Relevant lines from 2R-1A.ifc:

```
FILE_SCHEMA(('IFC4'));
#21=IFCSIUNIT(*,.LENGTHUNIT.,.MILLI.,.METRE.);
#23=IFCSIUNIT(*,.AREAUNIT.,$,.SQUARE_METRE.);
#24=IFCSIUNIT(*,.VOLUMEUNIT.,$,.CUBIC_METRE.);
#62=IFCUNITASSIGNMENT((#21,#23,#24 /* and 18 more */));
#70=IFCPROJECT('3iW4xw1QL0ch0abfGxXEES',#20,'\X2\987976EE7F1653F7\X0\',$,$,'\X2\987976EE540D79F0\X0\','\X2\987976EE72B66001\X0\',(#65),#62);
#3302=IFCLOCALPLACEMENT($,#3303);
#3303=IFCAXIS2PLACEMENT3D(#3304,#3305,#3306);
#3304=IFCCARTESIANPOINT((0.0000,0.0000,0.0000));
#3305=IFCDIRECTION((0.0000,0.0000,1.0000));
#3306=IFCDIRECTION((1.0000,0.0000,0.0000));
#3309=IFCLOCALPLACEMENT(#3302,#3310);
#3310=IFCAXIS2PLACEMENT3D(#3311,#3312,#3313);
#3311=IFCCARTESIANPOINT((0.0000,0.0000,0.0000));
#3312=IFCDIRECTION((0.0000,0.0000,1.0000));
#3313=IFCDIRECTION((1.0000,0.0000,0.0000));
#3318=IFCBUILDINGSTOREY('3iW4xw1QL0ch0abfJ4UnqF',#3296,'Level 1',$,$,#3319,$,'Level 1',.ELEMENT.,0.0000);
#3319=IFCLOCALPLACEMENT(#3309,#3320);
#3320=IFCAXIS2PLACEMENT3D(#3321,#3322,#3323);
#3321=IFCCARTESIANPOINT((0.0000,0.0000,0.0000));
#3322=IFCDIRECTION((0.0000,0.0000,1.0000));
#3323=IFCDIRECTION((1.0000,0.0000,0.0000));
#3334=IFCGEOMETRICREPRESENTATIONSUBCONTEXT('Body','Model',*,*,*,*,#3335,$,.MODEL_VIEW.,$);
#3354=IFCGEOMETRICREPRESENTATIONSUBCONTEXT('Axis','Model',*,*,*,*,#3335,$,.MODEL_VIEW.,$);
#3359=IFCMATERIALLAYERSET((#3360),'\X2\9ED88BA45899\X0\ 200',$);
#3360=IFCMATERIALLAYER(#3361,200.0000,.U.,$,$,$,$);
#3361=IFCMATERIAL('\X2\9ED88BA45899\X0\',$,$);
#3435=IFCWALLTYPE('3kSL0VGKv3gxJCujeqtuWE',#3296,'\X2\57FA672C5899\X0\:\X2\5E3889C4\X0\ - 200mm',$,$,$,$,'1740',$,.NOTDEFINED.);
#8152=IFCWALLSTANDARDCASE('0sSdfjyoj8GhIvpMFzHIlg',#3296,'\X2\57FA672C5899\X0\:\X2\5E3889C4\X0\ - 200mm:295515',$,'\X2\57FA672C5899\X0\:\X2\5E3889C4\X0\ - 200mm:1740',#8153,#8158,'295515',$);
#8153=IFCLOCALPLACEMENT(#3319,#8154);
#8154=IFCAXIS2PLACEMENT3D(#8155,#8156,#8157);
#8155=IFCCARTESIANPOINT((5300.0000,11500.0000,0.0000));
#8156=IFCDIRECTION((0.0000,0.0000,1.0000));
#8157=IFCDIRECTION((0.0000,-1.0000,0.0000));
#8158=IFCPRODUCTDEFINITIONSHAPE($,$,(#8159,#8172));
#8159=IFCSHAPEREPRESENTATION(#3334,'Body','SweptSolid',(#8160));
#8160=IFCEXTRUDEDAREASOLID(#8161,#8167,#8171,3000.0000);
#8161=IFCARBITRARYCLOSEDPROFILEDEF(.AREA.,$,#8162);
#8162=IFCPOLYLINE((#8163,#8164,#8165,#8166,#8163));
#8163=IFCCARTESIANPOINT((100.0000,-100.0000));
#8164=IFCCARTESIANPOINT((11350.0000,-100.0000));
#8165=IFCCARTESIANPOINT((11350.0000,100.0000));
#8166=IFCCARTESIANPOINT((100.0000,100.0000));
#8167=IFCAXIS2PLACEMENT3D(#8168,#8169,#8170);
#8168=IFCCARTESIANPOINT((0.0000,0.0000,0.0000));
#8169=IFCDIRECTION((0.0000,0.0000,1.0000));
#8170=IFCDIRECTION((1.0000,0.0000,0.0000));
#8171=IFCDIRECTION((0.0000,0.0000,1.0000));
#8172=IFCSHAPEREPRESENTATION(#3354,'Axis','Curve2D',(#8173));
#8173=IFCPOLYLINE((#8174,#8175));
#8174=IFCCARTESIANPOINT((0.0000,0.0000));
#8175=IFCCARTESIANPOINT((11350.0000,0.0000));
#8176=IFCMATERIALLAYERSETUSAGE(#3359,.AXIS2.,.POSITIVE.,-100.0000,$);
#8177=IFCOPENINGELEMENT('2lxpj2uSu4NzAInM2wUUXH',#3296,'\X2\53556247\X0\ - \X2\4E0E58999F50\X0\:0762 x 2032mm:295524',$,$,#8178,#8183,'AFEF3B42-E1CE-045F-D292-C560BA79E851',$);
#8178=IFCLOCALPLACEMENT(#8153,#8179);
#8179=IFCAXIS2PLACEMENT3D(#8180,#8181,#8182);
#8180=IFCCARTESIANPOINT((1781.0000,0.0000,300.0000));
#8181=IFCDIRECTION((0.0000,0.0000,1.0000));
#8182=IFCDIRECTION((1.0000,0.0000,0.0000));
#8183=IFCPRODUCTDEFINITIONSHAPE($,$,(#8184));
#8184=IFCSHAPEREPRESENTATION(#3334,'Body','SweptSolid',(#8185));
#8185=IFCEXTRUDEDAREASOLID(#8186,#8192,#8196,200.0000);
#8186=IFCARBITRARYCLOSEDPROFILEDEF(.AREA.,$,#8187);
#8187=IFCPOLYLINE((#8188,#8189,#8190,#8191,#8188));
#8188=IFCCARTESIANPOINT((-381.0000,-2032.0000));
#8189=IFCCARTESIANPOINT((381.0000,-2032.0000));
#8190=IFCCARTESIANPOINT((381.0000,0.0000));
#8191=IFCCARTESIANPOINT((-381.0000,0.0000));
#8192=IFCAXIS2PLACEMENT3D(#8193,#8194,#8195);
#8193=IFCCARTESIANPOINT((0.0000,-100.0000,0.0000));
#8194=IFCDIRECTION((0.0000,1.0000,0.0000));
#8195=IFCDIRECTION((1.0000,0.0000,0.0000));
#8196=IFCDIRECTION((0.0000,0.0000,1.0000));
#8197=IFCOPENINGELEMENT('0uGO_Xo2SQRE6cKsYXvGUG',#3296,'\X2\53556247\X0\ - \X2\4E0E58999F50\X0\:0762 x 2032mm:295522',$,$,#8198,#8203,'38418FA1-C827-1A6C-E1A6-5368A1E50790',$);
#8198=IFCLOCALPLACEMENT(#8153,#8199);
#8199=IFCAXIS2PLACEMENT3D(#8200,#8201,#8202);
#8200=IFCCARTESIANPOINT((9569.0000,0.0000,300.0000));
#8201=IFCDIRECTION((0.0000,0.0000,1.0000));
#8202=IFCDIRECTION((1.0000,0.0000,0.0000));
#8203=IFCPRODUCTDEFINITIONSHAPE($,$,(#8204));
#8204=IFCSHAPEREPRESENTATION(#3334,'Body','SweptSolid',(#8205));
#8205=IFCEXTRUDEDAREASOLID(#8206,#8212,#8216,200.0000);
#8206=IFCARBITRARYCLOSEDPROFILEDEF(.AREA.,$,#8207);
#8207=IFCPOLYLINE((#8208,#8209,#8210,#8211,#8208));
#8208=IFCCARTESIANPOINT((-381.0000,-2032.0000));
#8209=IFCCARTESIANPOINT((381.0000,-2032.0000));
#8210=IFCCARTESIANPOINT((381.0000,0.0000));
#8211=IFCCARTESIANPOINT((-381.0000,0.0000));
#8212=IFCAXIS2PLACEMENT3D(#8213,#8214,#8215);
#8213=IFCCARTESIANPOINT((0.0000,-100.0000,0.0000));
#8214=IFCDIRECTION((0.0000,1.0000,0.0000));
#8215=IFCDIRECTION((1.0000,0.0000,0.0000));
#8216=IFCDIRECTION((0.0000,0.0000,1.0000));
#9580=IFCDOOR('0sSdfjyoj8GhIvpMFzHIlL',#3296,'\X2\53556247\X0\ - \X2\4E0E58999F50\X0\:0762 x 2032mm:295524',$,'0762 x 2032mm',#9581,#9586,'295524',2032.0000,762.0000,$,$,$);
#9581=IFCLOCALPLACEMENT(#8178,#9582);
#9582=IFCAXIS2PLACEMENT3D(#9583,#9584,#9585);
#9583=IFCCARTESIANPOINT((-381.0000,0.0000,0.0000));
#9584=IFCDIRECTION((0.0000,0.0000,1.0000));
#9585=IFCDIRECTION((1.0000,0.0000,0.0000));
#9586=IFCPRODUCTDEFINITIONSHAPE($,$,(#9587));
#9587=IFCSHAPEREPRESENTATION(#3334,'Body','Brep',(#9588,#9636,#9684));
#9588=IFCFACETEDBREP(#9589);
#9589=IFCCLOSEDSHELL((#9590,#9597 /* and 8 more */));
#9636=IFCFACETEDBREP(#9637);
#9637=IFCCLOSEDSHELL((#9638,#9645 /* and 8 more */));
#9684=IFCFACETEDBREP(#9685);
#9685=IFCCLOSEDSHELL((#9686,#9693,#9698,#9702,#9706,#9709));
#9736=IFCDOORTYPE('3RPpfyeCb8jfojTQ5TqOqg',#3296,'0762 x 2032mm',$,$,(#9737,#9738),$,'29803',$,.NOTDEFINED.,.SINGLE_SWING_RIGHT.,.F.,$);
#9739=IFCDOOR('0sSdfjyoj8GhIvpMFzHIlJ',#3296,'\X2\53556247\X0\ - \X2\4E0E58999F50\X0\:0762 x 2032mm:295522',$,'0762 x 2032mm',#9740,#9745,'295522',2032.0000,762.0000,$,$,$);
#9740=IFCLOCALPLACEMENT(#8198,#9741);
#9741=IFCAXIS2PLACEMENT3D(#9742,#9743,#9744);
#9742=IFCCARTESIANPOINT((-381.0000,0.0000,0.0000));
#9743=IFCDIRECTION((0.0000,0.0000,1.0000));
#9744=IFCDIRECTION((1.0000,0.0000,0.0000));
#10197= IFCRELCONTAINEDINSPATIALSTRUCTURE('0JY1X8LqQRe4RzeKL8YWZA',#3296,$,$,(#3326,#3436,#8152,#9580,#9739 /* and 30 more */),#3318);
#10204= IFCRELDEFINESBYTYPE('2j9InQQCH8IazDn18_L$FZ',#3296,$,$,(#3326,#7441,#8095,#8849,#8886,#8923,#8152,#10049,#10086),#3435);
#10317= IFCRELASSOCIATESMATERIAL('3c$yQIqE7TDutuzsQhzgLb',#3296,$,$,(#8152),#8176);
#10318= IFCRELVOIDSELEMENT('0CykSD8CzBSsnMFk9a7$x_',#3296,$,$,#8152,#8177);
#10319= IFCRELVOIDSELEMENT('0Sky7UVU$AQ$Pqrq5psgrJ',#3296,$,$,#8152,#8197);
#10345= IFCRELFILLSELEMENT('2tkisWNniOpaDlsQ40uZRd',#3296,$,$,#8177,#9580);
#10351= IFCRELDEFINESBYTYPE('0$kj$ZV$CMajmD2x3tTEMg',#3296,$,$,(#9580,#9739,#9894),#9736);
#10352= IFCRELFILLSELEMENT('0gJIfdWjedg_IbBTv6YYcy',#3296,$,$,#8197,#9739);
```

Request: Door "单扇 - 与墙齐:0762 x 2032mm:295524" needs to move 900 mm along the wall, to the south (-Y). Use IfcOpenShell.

```python
import ifcopenshell
import ifcopenshell.api.geometry
import ifcopenshell.util.placement

model = ifcopenshell.open("2R-1A.ifc")

door = model.by_guid("0sSdfjyoj8GhIvpMFzHIlL")
opening = door.FillsVoids[0].RelatingOpeningElement
wall = opening.VoidsElements[0].RelatingBuildingElement

wall_matrix = ifcopenshell.util.placement.get_local_placement(wall.ObjectPlacement)
shift = wall_matrix[:3, 0] * 900.0
before = ifcopenshell.util.placement.get_local_placement(door.ObjectPlacement)[:3, 3].copy()

# The door is placed relative to its opening, so it follows when the opening moves.
matrix = ifcopenshell.util.placement.get_local_placement(opening.ObjectPlacement)
matrix[:3, 3] += shift
ifcopenshell.api.geometry.edit_object_placement(
    model, product=opening, matrix=matrix, is_si=False, should_transform_children=True
)

after = ifcopenshell.util.placement.get_local_placement(door.ObjectPlacement)[:3, 3]
print("door moved by", (after - before).round(3) + 0.0)

model.write("2R-1A_updated.ifc")
```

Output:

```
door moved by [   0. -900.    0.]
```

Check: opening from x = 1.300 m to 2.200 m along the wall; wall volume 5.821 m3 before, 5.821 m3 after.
